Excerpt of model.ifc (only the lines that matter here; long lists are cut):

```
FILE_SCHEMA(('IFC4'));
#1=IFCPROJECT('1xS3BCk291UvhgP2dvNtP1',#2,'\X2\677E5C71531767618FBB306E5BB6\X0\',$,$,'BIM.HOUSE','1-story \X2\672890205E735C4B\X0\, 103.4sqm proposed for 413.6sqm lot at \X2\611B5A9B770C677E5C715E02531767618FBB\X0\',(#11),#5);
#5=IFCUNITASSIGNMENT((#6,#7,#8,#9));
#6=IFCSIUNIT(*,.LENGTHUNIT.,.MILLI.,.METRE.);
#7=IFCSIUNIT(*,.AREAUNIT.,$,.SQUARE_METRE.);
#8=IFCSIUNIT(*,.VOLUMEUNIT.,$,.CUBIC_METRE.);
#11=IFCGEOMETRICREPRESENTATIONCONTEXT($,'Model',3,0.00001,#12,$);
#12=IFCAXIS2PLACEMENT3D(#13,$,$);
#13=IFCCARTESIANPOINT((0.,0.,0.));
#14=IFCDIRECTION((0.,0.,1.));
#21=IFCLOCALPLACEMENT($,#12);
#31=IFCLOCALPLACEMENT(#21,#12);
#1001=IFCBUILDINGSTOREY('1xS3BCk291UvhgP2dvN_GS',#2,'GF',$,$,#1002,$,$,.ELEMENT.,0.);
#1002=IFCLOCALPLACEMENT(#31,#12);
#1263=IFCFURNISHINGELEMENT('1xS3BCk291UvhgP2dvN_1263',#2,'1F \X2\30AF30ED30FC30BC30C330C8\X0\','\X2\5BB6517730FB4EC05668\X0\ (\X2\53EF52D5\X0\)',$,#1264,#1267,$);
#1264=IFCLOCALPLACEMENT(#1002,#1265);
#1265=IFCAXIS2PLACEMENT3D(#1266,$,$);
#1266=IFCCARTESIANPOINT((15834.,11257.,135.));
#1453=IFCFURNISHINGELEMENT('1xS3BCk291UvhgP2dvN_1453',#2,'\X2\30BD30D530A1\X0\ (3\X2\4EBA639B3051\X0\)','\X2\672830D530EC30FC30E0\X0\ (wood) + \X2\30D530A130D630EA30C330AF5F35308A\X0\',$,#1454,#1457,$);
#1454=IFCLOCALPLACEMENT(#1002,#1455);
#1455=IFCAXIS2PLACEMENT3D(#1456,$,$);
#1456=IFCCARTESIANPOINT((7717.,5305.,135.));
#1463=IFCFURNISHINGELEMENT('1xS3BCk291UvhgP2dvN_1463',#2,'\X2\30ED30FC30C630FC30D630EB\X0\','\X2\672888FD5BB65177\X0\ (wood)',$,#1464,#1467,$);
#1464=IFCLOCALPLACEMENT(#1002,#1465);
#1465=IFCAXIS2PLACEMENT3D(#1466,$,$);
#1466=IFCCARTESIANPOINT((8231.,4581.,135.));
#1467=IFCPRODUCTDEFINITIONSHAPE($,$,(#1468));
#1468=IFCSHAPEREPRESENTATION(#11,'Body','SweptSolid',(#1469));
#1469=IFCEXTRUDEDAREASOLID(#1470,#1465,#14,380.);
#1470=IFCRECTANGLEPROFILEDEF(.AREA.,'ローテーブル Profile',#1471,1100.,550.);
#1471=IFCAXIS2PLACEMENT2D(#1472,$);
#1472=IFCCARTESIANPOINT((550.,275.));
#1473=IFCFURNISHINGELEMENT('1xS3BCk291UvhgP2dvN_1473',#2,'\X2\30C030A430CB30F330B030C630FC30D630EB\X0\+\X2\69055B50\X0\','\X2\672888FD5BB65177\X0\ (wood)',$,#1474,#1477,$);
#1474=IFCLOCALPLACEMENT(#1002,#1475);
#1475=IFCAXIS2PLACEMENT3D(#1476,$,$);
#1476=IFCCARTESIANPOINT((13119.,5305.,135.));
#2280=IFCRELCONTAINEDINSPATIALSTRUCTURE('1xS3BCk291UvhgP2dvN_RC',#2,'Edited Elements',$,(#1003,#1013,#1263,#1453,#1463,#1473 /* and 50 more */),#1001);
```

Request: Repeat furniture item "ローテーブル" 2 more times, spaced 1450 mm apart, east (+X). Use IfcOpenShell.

```python
import numpy as np
import ifcopenshell
import ifcopenshell.api.geometry
import ifcopenshell.api.root
import ifcopenshell.util.element
import ifcopenshell.util.placement

model = ifcopenshell.open("model.ifc")


def reuse_history(source, copy):
    """copy_class also copies each property set's owner history, people and application; keep the originals."""
    for rel in copy.IsDefinedBy:
        if rel.is_a("IfcRelDefinesByProperties") and (history := rel.RelatingPropertyDefinition.OwnerHistory):
            rel.RelatingPropertyDefinition.OwnerHistory = source.OwnerHistory
            ifcopenshell.util.element.remove_deep2(model, history)


source = model.by_guid("1xS3BCk291UvhgP2dvN_1463")
base = ifcopenshell.util.placement.get_local_placement(source.ObjectPlacement)
step = np.array([1.0, 0.0, 0.0]) * 1450.0

for i in range(1, 3):
    copy = ifcopenshell.api.root.copy_class(model, product=source)
    copy.Representation = ifcopenshell.util.element.copy_deep(
        model, source.Representation, exclude=["IfcGeometricRepresentationContext", "IfcRepresentationMap"]
    )
    reuse_history(source, copy)
    matrix = base.copy()
    matrix[:3, 3] += i * step
    print("added at", matrix[:3, 3].round(3) + 0.0)
    ifcopenshell.api.geometry.edit_object_placement(model, product=copy, matrix=matrix, is_si=False)

model.write("model_v2.ifc")
```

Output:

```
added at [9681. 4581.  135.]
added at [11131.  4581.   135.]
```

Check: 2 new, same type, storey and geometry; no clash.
